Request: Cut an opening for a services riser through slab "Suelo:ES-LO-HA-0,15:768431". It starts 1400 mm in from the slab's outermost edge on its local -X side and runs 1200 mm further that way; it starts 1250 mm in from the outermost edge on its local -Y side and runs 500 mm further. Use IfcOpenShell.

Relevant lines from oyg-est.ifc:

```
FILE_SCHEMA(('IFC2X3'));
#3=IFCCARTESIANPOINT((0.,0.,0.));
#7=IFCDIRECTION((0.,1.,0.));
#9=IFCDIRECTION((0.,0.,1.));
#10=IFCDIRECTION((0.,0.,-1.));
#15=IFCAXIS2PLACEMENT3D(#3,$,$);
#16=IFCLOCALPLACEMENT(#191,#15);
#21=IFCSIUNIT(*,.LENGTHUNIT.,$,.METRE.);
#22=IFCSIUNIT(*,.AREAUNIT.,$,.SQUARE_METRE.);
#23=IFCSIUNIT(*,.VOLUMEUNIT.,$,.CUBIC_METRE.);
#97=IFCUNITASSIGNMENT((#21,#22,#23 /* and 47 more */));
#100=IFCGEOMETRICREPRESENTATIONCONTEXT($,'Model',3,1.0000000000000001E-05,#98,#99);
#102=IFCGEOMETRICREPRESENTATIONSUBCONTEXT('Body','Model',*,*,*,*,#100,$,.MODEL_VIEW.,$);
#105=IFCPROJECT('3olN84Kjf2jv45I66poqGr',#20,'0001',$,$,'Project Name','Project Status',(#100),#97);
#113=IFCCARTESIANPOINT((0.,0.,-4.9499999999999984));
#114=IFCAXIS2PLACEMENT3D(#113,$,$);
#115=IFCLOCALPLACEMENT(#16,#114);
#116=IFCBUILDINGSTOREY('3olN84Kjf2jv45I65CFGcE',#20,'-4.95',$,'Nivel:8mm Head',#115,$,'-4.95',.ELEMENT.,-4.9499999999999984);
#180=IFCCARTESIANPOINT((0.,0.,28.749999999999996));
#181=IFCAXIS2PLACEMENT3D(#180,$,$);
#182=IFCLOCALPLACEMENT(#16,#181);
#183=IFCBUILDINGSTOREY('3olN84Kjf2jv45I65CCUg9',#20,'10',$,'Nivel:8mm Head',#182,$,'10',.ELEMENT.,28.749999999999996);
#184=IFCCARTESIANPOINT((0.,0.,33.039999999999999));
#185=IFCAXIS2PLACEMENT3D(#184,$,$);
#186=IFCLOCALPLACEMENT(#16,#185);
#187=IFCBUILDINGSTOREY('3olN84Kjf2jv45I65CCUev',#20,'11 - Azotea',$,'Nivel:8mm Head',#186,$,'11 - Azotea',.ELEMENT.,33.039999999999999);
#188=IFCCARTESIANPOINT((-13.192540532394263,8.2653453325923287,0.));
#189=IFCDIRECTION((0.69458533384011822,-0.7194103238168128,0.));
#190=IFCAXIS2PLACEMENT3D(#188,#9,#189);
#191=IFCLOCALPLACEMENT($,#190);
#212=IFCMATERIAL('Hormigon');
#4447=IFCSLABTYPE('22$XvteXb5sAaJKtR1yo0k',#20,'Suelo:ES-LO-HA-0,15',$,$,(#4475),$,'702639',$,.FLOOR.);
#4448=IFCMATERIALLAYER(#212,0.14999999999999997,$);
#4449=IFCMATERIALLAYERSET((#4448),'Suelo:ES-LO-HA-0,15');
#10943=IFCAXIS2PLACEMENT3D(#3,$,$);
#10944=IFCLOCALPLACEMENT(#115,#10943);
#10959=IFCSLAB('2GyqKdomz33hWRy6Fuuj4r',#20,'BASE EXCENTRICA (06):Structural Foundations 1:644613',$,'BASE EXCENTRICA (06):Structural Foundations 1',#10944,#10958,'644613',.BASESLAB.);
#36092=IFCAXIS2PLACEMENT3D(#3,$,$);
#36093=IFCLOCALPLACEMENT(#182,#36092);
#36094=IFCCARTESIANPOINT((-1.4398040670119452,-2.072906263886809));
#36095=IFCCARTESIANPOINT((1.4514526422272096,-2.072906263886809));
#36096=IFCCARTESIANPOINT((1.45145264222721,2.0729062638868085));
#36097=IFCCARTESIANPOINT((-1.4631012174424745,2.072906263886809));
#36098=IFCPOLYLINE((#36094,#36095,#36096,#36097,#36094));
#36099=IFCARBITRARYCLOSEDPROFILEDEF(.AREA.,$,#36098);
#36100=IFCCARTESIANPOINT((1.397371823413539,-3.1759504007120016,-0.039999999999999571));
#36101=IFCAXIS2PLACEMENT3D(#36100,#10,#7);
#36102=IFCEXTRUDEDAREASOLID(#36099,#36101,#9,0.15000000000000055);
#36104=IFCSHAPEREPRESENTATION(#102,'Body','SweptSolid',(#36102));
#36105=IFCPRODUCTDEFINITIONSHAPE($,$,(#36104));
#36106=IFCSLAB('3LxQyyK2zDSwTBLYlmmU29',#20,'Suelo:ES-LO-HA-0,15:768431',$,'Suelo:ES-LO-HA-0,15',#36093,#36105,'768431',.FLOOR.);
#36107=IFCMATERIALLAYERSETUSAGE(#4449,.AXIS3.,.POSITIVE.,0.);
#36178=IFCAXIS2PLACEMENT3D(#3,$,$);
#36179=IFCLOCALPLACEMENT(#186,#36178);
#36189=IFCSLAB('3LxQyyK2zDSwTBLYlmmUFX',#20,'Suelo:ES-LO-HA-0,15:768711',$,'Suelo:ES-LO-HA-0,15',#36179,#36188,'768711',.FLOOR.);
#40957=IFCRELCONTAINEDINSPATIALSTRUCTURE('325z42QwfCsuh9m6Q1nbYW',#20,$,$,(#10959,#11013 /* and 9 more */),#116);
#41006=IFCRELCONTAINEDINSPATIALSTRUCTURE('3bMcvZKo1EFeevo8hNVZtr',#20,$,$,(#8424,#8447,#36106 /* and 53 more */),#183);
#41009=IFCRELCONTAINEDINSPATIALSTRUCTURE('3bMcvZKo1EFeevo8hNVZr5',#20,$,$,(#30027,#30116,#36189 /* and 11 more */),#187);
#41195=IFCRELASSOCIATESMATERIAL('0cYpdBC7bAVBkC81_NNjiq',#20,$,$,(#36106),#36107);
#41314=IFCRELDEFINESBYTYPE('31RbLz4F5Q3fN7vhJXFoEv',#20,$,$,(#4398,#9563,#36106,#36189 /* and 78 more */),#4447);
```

```python
import numpy as np
import ifcopenshell
import ifcopenshell.api.feature
import ifcopenshell.api.geometry
import ifcopenshell.api.root
import ifcopenshell.geom
import ifcopenshell.util.placement
import ifcopenshell.util.representation
import ifcopenshell.util.shape
import ifcopenshell.util.unit

model = ifcopenshell.open("oyg-est.ifc")
unit_scale = ifcopenshell.util.unit.calculate_unit_scale(model)
settings = ifcopenshell.geom.settings()


def volume(element):
    """Net volume in cubic metres, openings subtracted."""
    shape = ifcopenshell.geom.create_shape(settings, element)
    return ifcopenshell.util.shape.get_volume(shape.geometry)


slab = model.by_id(36106)
before = volume(slab)

# Extent in the slab's own axes, in metres. The edges named are its -X and -Y sides.
slab_shape = ifcopenshell.geom.create_shape(settings, slab)
vertices = ifcopenshell.util.shape.get_vertices(slab_shape.geometry)
x_min, y_min, bottom = vertices.min(axis=0)
top = vertices[:, 2].max()

opening = ifcopenshell.api.root.create_entity(model, ifc_class="IfcOpeningElement", name="Services riser opening")
context = ifcopenshell.util.representation.get_context(model, "Model", "Body", "MODEL_VIEW")
width, depth = 1.2, 0.5
outline = [(0.0, 0.0), (width, 0.0), (width, depth), (0.0, depth), (0.0, 0.0)]
# Overshoot both faces by 50 mm so the cut is clean.
shape = ifcopenshell.api.geometry.add_slab_representation(
    model, context=context, depth=top - bottom + 0.1, polyline=outline
)
ifcopenshell.api.geometry.assign_representation(model, product=opening, representation=shape)

matrix = ifcopenshell.util.placement.get_local_placement(slab.ObjectPlacement)
matrix[:, 3] = matrix @ np.append(np.array([x_min + 1.4, y_min + 1.25, bottom - 0.05]) / unit_scale, 1.0)
ifcopenshell.api.geometry.edit_object_placement(model, product=opening, matrix=matrix, is_si=False)
ifcopenshell.api.feature.add_feature(model, feature=opening, element=slab)

after = volume(slab)

print(f"slab volume {before:.3f} -> {after:.3f} m3")

model.write("oyg-est_rev.ifc")
```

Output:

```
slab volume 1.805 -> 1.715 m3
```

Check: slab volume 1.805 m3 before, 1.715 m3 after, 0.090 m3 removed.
